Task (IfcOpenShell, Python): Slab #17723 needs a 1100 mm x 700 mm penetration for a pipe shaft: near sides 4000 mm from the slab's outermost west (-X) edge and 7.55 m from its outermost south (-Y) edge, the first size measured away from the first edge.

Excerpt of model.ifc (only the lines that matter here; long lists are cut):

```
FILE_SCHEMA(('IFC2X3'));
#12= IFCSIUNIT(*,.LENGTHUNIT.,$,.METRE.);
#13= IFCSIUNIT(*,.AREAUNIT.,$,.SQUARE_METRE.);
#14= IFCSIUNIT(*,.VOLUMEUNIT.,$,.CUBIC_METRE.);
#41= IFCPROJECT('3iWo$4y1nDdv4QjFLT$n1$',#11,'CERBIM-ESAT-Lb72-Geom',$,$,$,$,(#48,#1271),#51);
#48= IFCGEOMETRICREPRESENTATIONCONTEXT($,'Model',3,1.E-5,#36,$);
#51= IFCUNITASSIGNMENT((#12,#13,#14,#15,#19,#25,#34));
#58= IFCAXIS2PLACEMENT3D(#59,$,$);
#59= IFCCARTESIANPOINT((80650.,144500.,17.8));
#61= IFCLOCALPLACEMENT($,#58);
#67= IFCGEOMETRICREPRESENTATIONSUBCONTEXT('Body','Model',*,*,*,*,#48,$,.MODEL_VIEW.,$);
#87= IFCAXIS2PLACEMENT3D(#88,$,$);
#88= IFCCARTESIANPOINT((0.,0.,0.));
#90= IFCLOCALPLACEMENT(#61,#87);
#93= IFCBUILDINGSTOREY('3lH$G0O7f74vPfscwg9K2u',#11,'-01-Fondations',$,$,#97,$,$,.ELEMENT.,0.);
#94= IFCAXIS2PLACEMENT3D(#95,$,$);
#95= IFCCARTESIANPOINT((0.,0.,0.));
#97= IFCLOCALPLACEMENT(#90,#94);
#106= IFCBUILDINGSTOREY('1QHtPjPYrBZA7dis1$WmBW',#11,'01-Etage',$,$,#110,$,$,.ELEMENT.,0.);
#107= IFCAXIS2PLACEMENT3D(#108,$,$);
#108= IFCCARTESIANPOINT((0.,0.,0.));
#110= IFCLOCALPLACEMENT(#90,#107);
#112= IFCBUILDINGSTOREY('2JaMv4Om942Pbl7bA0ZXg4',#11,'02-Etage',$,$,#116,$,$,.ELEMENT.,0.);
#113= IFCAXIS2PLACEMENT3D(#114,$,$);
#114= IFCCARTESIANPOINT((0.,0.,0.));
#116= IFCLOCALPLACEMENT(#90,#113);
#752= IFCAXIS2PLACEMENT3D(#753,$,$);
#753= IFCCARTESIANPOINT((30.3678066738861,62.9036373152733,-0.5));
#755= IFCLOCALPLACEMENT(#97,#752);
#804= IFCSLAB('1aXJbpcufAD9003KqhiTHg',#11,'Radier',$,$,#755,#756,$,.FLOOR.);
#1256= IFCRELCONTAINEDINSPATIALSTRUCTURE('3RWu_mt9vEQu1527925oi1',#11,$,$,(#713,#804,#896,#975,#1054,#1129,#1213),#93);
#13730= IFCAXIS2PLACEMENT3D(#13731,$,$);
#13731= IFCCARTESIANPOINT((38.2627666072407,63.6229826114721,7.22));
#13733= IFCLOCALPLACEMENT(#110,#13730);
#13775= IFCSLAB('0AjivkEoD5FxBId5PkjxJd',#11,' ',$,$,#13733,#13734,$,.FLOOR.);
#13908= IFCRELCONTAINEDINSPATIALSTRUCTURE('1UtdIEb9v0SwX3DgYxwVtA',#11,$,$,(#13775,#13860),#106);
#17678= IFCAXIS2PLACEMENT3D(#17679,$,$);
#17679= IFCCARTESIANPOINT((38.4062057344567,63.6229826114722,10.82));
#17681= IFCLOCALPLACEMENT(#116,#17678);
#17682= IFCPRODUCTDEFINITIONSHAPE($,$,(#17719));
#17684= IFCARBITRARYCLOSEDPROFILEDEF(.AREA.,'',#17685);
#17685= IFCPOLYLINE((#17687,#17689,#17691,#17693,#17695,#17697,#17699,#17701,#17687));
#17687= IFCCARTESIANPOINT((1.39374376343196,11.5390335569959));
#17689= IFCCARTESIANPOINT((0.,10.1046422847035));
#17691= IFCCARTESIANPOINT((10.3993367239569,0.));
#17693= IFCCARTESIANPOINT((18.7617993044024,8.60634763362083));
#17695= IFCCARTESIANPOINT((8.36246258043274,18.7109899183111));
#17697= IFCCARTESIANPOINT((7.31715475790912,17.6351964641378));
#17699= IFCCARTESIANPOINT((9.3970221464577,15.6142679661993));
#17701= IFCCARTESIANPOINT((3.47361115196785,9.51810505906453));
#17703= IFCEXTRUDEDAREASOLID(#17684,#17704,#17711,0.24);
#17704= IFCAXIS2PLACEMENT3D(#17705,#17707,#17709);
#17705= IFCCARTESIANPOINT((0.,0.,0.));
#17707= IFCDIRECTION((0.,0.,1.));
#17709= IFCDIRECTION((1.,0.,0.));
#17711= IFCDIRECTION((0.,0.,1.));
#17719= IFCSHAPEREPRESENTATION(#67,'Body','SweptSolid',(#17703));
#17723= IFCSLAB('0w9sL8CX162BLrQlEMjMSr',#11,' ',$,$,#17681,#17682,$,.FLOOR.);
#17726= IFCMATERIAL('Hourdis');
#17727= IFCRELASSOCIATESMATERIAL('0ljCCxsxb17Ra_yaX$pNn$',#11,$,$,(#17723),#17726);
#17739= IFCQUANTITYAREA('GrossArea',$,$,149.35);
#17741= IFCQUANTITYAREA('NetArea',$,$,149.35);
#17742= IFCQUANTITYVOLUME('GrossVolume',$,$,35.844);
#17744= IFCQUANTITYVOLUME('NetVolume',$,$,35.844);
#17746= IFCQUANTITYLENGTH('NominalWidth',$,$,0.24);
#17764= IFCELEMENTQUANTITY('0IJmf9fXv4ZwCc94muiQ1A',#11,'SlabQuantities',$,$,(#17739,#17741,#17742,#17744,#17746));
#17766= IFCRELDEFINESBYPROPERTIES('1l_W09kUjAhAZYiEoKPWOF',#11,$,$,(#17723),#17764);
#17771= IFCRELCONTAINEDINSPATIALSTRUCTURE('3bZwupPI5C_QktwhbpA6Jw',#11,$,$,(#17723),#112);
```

```python
import numpy as np
import ifcopenshell
import ifcopenshell.api.feature
import ifcopenshell.api.geometry
import ifcopenshell.api.pset
import ifcopenshell.api.root
import ifcopenshell.geom
import ifcopenshell.util.element
import ifcopenshell.util.placement
import ifcopenshell.util.representation
import ifcopenshell.util.shape
import ifcopenshell.util.unit

model = ifcopenshell.open("model.ifc")
unit_scale = ifcopenshell.util.unit.calculate_unit_scale(model)
area_scale = ifcopenshell.util.unit.calculate_unit_scale(model, "AREAUNIT")
volume_scale = ifcopenshell.util.unit.calculate_unit_scale(model, "VOLUMEUNIT")
settings = ifcopenshell.geom.settings()


def volume(element):
    """Net volume in cubic metres, openings subtracted."""
    shape = ifcopenshell.geom.create_shape(settings, element)
    return ifcopenshell.util.shape.get_volume(shape.geometry)


slab = model.by_guid("0w9sL8CX162BLrQlEMjMSr")
before = volume(slab)

# Extent in the slab's own axes, in metres. The edges named are its -X and -Y sides.
slab_shape = ifcopenshell.geom.create_shape(settings, slab)
vertices = ifcopenshell.util.shape.get_vertices(slab_shape.geometry)
x_min, y_min, bottom = vertices.min(axis=0)
top = vertices[:, 2].max()

opening = ifcopenshell.api.root.create_entity(model, ifc_class="IfcOpeningElement", name="Pipe shaft opening")
context = ifcopenshell.util.representation.get_context(model, "Model", "Body", "MODEL_VIEW")
width, depth = 1.1, 0.7
outline = [(0.0, 0.0), (width, 0.0), (width, depth), (0.0, depth), (0.0, 0.0)]
# Overshoot both faces by 50 mm so the cut is clean.
shape = ifcopenshell.api.geometry.add_slab_representation(
    model, context=context, depth=top - bottom + 0.1, polyline=outline
)
ifcopenshell.api.geometry.assign_representation(model, product=opening, representation=shape)

matrix = ifcopenshell.util.placement.get_local_placement(slab.ObjectPlacement)
matrix[:, 3] = matrix @ np.append(np.array([x_min + 4, y_min + 7.55, bottom - 0.05]) / unit_scale, 1.0)
ifcopenshell.api.geometry.edit_object_placement(model, product=opening, matrix=matrix, is_si=False)
ifcopenshell.api.feature.add_feature(model, feature=opening, element=slab)

after = volume(slab)

# Update the slab's stored quantities.
qto = model.by_id(ifcopenshell.util.element.get_pset(slab, "SlabQuantities", should_inherit=False)["id"])
ifcopenshell.api.pset.edit_qto(model, qto=qto, properties={
    "NetArea": after / (top - bottom) / area_scale,
    "NetVolume": after / volume_scale,
})

print(f"slab volume {before:.3f} -> {after:.3f} m3")

model.write("model_rev.ifc")
```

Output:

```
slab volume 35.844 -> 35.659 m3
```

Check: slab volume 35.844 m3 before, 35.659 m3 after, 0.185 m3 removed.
